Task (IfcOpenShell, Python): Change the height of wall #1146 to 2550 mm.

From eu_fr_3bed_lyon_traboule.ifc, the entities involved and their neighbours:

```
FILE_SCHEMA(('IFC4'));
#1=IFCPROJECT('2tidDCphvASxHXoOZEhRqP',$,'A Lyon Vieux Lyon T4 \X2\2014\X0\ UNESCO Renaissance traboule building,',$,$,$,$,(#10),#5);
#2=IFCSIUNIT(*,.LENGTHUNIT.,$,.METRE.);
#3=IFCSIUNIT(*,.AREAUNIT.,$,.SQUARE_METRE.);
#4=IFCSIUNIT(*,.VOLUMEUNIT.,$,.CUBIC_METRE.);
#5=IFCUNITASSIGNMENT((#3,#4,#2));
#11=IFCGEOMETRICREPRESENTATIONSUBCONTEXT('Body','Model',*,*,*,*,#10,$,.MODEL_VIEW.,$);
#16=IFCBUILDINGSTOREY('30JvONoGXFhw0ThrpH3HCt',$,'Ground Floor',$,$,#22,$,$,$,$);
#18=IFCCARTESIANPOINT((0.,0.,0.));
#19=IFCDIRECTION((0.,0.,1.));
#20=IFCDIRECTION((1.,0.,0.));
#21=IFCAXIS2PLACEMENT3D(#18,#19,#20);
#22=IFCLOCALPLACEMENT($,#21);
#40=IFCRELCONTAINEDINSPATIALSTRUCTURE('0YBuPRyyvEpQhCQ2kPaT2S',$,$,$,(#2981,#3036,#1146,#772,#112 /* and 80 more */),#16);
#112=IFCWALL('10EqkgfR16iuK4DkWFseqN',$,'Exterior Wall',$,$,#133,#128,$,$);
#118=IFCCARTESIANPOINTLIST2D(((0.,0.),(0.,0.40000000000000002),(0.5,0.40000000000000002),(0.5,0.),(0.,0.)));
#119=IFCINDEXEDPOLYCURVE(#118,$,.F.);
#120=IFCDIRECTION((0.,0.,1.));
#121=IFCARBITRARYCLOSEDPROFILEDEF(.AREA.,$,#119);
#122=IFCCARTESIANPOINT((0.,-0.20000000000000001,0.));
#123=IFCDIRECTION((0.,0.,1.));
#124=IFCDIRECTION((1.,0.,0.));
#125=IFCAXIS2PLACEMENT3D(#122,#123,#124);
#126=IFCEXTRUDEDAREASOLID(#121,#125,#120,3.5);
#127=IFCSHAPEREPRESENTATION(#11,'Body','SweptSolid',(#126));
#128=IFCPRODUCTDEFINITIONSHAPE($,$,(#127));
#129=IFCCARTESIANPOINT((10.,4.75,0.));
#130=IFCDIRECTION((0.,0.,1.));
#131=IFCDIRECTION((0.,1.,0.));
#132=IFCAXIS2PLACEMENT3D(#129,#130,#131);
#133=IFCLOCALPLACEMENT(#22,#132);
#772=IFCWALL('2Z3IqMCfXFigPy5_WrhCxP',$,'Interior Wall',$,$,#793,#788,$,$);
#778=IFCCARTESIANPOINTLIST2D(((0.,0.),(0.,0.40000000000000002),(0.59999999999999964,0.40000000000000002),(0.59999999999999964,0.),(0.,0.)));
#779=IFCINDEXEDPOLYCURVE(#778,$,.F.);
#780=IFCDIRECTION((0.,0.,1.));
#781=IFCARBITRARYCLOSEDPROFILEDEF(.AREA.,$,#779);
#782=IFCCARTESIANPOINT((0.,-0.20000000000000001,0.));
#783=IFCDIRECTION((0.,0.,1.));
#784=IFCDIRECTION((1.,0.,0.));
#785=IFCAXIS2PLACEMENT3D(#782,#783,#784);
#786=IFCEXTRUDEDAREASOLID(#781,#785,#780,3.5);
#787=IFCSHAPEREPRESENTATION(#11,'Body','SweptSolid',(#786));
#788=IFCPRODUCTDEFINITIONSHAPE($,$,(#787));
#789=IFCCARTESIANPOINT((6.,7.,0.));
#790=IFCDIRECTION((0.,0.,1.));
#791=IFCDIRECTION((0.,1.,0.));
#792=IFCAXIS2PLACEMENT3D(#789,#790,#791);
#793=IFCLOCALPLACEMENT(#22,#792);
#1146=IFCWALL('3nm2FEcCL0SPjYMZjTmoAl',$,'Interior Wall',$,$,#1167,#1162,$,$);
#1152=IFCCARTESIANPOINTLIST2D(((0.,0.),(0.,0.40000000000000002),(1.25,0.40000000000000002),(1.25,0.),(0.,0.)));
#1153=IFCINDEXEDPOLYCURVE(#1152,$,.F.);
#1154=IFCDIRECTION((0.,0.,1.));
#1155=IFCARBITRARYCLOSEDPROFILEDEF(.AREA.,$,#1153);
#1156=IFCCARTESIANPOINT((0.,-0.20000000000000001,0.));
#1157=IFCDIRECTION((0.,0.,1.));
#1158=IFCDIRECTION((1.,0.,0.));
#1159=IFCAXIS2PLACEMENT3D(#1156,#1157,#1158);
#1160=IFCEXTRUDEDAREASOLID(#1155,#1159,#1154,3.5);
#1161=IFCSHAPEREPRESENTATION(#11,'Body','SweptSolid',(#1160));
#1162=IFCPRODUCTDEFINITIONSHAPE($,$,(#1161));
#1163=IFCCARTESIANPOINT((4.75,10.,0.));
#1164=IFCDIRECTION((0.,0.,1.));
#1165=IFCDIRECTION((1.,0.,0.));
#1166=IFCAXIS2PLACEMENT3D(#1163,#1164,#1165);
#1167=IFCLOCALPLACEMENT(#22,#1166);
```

```python
import ifcopenshell
import ifcopenshell.geom
import ifcopenshell.util.representation
import ifcopenshell.util.shape
import ifcopenshell.util.unit

model = ifcopenshell.open("eu_fr_3bed_lyon_traboule.ifc")
unit_scale = ifcopenshell.util.unit.calculate_unit_scale(model)
settings = ifcopenshell.geom.settings()


def volume(element):
    """Net volume in cubic metres, openings subtracted."""
    shape = ifcopenshell.geom.create_shape(settings, element)
    return ifcopenshell.util.shape.get_volume(shape.geometry)


wall = model.by_id(1146)
before = volume(wall)

body = ifcopenshell.util.representation.get_representation(wall, "Model", "Body")
solid = body.Items[0]
old_height = solid.Depth
solid.Depth = 2.55 / unit_scale
after = volume(wall)

print(f"height {old_height:g} -> {solid.Depth:g}, volume {before:.3f} -> {after:.3f} m3")

model.write("eu_fr_3bed_lyon_traboule_v2.ifc")
```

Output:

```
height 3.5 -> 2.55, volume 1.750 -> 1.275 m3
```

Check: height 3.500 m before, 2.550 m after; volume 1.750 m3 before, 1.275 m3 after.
